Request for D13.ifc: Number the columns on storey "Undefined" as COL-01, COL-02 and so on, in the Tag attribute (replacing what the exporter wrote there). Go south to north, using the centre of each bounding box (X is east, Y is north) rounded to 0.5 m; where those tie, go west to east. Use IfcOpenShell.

First a look at what the model holds.

```python
import ifcopenshell
import ifcopenshell.util.element
import ifcopenshell.util.placement

model = ifcopenshell.open("D13.ifc")
print(model.schema)
storey = next(s for s in model.by_type("IfcBuildingStorey") if s.Name == "Undefined")
columns = [e for e in ifcopenshell.util.element.get_decomposition(storey) if e.is_a("IfcColumn")]
for e in sorted(columns, key=lambda e: e.id()):
    origin = ifcopenshell.util.placement.get_local_placement(e.ObjectPlacement)[:3, 3]
    print(e.id(), e.Tag, e.Name, origin.round(2) + 0.0, sep=" | ")
```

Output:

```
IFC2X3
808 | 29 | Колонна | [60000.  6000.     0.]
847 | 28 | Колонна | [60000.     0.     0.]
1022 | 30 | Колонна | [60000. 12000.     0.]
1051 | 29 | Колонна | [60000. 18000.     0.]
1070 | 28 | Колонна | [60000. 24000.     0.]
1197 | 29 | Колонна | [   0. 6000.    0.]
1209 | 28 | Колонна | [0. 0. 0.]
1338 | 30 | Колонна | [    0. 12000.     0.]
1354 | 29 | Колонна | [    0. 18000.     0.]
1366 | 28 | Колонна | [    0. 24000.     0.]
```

```python
import ifcopenshell
import ifcopenshell.geom
import ifcopenshell.util.element
import ifcopenshell.util.shape

model = ifcopenshell.open("D13.ifc")
settings = ifcopenshell.geom.settings()
settings.set("use-world-coords", True)


def centre(element):
    shape = ifcopenshell.geom.create_shape(settings, element)
    return ifcopenshell.util.shape.get_bbox_centroid(shape.geometry)


storey = next(s for s in model.by_type("IfcBuildingStorey") if s.Name == "Undefined")
columns = [e for e in ifcopenshell.util.element.get_decomposition(storey) if e.is_a("IfcColumn")]

# Insertion points can sit at a corner or the storey origin, so sort by the geometry (in metres).
centres = {e: centre(e) for e in columns}
columns.sort(key=lambda e: (round(centres[e][1] / 0.5), centres[e][0]))

for i, e in enumerate(columns, start=1):
    number = f"COL-{i:02d}"
    e.Tag = number
    print(e.id(), number)

model.write("D13-out.ifc")
```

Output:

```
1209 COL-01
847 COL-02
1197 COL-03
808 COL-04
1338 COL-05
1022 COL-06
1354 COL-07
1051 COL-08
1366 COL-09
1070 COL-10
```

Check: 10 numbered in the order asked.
